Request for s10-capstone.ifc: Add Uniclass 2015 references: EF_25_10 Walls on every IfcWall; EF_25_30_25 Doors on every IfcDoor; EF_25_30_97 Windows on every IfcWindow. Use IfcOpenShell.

First a look at what the model holds.

```python
import ifcopenshell

model = ifcopenshell.open("s10-capstone.ifc")
print(model.schema)
print("classifications:", [c.Name for c in model.by_type("IfcClassification")])
for ifc_class in ("IfcDoor", "IfcRoof", "IfcStair", "IfcWall", "IfcWindow"):
    print(ifc_class, len(model.by_type(ifc_class)))
```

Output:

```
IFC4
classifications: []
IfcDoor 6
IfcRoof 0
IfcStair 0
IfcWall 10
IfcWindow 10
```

```python
import ifcopenshell
import ifcopenshell.api.classification

model = ifcopenshell.open("s10-capstone.ifc")

system = ifcopenshell.api.classification.add_classification(model, classification="Uniclass 2015")

codes = {
    "IfcWall": ("EF_25_10", "Walls"),
    "IfcDoor": ("EF_25_30_25", "Doors"),
    "IfcWindow": ("EF_25_30_97", "Windows"),
}
for ifc_class, (code, name) in codes.items():
    products = model.by_type(ifc_class)
    ifcopenshell.api.classification.add_reference(
        model, products=products, classification=system, identification=code, name=name
    )
    print(code, len(products))

model.write("s10-capstone-out.ifc")
```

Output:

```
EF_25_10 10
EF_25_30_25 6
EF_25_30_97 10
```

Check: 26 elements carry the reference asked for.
